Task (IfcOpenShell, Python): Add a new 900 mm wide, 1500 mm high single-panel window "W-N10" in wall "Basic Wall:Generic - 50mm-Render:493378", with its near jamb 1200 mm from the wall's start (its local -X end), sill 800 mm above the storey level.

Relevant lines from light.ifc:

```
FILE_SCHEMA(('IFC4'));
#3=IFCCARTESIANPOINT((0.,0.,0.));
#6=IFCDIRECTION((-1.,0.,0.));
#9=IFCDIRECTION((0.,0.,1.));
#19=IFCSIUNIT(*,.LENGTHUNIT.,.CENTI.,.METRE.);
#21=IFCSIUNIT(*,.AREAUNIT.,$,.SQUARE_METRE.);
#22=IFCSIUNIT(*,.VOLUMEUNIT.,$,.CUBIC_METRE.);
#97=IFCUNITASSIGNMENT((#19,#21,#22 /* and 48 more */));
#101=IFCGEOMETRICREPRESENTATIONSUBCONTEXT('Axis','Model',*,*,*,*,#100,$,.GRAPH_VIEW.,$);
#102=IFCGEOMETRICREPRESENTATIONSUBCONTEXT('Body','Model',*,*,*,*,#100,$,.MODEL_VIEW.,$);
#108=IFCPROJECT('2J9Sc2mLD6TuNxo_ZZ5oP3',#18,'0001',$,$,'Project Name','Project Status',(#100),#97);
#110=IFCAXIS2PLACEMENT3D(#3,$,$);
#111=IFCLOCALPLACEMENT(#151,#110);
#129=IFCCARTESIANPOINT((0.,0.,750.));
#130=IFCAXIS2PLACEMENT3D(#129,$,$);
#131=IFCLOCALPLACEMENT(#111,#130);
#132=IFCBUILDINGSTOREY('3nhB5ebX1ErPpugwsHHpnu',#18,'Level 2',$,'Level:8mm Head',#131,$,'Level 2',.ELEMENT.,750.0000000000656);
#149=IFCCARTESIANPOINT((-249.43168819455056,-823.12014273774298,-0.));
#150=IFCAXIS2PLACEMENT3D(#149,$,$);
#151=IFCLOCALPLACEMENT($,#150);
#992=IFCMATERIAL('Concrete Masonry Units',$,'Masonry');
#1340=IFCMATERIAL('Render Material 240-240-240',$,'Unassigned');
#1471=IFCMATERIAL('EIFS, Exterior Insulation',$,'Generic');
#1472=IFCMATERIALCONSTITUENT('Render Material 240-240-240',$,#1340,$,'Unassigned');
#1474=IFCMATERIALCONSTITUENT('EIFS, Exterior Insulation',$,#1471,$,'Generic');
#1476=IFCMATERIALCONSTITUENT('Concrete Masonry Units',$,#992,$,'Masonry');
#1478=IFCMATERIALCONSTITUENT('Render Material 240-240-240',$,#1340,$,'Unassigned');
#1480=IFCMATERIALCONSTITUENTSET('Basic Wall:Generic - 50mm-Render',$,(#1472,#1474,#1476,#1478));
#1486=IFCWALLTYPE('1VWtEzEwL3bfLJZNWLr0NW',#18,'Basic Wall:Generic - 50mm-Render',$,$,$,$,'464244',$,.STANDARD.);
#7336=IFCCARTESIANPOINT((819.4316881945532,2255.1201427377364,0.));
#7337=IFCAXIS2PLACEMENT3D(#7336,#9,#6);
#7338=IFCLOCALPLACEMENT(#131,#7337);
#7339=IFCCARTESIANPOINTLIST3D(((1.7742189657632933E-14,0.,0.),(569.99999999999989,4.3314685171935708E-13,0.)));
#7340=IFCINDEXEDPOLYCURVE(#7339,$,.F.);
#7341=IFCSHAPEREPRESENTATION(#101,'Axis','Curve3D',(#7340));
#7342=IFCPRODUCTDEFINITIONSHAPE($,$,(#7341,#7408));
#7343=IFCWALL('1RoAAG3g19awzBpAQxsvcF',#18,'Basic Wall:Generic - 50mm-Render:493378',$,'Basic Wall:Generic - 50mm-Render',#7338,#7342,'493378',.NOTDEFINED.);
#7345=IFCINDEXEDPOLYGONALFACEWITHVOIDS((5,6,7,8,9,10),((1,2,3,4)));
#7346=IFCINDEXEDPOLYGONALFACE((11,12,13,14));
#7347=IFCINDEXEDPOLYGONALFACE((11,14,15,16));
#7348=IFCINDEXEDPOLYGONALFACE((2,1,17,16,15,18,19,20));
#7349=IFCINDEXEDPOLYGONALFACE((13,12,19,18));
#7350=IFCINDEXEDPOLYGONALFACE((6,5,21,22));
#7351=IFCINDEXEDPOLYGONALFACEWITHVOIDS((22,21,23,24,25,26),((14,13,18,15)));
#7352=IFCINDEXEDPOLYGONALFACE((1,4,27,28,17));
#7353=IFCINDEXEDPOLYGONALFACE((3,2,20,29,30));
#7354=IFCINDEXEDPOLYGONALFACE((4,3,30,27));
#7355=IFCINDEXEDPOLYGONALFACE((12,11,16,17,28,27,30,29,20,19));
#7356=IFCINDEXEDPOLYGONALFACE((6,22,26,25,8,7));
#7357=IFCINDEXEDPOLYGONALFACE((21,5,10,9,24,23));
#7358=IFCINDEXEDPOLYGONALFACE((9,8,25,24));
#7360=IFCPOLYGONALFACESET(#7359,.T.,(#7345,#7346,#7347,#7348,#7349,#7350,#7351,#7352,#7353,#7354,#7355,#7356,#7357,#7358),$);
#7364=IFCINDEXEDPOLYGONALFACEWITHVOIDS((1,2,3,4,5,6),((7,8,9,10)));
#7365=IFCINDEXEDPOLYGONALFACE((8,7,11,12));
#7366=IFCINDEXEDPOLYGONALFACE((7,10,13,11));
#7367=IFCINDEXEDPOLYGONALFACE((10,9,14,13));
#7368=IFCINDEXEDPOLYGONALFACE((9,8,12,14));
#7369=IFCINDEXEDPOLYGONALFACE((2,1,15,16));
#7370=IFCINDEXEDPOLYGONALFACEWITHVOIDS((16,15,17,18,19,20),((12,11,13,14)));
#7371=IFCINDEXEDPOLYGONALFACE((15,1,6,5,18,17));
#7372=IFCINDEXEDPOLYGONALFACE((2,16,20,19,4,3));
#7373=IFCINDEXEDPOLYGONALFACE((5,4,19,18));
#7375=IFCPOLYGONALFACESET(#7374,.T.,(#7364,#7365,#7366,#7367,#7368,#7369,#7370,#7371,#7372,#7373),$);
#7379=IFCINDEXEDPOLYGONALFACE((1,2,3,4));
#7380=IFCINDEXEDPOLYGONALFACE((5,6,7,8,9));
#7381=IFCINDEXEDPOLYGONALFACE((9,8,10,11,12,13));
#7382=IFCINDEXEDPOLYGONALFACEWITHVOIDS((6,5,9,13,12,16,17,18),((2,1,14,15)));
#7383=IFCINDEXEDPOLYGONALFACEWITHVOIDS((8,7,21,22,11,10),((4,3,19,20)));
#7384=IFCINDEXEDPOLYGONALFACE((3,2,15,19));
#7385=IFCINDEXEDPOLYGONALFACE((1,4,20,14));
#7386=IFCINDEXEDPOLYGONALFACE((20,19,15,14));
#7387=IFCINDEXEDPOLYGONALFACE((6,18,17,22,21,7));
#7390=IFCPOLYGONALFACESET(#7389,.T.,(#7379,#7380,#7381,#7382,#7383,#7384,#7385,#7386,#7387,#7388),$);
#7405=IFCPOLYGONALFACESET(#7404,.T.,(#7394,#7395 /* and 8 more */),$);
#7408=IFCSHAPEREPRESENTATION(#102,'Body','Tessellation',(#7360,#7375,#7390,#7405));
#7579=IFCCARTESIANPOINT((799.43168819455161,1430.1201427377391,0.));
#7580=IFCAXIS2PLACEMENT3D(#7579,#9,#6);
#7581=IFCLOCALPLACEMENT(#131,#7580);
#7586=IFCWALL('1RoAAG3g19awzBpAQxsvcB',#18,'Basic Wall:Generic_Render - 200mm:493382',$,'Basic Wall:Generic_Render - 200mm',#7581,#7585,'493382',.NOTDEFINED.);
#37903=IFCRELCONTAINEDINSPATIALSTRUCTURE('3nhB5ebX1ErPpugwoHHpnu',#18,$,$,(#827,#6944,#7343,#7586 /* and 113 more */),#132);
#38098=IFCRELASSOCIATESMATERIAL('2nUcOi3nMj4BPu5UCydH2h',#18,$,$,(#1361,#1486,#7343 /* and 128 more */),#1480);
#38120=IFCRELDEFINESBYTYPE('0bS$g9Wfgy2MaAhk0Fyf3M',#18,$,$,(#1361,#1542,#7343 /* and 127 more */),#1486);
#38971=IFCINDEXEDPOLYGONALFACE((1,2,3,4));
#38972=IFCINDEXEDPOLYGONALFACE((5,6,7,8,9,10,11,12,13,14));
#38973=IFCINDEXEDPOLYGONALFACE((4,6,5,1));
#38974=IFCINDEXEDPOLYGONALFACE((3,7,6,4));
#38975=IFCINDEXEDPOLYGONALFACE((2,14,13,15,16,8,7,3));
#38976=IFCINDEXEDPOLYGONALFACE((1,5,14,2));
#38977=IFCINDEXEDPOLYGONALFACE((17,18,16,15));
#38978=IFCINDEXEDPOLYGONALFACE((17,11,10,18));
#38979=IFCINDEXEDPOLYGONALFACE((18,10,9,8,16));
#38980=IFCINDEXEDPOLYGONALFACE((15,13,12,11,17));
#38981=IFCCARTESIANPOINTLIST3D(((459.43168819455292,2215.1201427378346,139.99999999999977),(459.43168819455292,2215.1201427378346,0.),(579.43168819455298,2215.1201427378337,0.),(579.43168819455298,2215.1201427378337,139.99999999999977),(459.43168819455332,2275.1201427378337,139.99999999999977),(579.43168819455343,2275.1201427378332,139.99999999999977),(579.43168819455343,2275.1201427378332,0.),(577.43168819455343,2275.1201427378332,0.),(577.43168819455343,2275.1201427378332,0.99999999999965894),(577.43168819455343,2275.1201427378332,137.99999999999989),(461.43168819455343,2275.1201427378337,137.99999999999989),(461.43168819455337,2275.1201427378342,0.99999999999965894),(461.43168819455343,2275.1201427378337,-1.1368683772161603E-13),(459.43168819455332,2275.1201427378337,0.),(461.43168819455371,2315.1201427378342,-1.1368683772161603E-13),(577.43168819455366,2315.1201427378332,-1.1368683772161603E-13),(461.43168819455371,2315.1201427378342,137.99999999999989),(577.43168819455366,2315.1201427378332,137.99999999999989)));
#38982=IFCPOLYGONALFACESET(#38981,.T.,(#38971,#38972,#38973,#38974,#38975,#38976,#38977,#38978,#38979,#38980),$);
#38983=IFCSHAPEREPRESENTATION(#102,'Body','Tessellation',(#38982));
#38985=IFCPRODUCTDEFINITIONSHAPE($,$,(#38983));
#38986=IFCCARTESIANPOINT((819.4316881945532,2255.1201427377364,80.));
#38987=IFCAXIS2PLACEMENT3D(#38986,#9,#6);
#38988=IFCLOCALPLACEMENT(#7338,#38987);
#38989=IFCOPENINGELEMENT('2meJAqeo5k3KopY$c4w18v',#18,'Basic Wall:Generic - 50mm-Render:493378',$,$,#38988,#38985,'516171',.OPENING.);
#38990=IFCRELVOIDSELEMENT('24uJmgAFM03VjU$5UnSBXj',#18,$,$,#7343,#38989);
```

```python
import numpy as np
import ifcopenshell
import ifcopenshell.api.feature
import ifcopenshell.api.geometry
import ifcopenshell.api.root
import ifcopenshell.api.spatial
import ifcopenshell.geom
import ifcopenshell.util.element
import ifcopenshell.util.placement
import ifcopenshell.util.representation
import ifcopenshell.util.shape
import ifcopenshell.util.unit

model = ifcopenshell.open("light.ifc")
unit_scale = ifcopenshell.util.unit.calculate_unit_scale(model)
settings = ifcopenshell.geom.settings()


def volume(element):
    """Net volume in cubic metres, openings subtracted."""
    shape = ifcopenshell.geom.create_shape(settings, element)
    return ifcopenshell.util.shape.get_volume(shape.geometry)


wall = model.by_guid("1RoAAG3g19awzBpAQxsvcF")
storey = ifcopenshell.util.element.get_container(wall, ifc_class="IfcBuildingStorey")
context = ifcopenshell.util.representation.get_context(model, "Model", "Body", "MODEL_VIEW")
before = volume(wall)

width, height, from_end, sill = 0.9, 1.5, 1.2, 0.8  # metres

# The wall runs along its own X axis, and the end named is its -X end.
wall_shape = ifcopenshell.geom.create_shape(settings, wall)
x, y, z = ifcopenshell.util.shape.get_vertices(wall_shape.geometry).T
start = x.min() + from_end
face, thickness = float(y.min()), float(y.max() - y.min())
wall_matrix = ifcopenshell.util.placement.get_local_placement(wall.ObjectPlacement)
level = ifcopenshell.util.placement.get_local_placement(storey.ObjectPlacement)[2, 3]


def in_wall(x, y):
    """Placement at x, y metres in the wall's axes, at sill height."""
    matrix = wall_matrix.copy()
    matrix[:, 3] = wall_matrix @ np.array([x / unit_scale, y / unit_scale, 0.0, 1.0])
    matrix[2, 3] = level + sill / unit_scale
    return matrix


# Opening: a box that overshoots both wall faces by 50 mm.
opening = ifcopenshell.api.root.create_entity(model, ifc_class="IfcOpeningElement", predefined_type="OPENING")
box = ifcopenshell.api.geometry.add_wall_representation(
    model, context=context, length=width, height=height, thickness=thickness + 0.1
)
ifcopenshell.api.geometry.assign_representation(model, product=opening, representation=box)
ifcopenshell.api.geometry.edit_object_placement(model, product=opening, matrix=in_wall(start, face - 0.05), is_si=False)
ifcopenshell.api.feature.add_feature(model, feature=opening, element=wall)

window = ifcopenshell.api.root.create_entity(model, ifc_class="IfcWindow", name="W-N10", predefined_type="WINDOW")
window.OverallWidth, window.OverallHeight = width / unit_scale, height / unit_scale
window.PartitioningType = "SINGLE_PANEL"
body = ifcopenshell.api.geometry.add_window_representation(
    model,
    context=context,
    overall_width=window.OverallWidth,
    overall_height=window.OverallHeight,
    partition_type="SINGLE_PANEL",
)
ifcopenshell.api.geometry.assign_representation(model, product=window, representation=body)
ifcopenshell.api.spatial.assign_container(model, products=[window], relating_structure=storey)
ifcopenshell.api.feature.add_filling(model, opening=opening, element=window)

# Centre the window in the wall's thickness.
ifcopenshell.api.geometry.edit_object_placement(model, product=window, matrix=in_wall(start, face), is_si=False)
window_shape = ifcopenshell.geom.create_shape(settings, window)
depth = ifcopenshell.util.shape.get_vertices(window_shape.geometry)[:, 1]
offset = face + thickness / 2 - (depth.min() + depth.max()) / 2
ifcopenshell.api.geometry.edit_object_placement(model, product=window, matrix=in_wall(start, offset), is_si=False)

after = volume(wall)

print(f"wall volume {before:.3f} -> {after:.3f} m3")

model.write("light_updated.ifc")
```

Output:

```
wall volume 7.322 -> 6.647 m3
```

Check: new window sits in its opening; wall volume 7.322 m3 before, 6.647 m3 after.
